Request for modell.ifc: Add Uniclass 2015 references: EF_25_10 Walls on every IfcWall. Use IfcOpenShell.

First a look at what the model holds.

```python
import ifcopenshell

model = ifcopenshell.open("modell.ifc")
print(model.schema)
print("classifications:", [c.Name for c in model.by_type("IfcClassification")])
for ifc_class in ("IfcDoor", "IfcRoof", "IfcStair", "IfcWall", "IfcWindow"):
    print(ifc_class, len(model.by_type(ifc_class)))
```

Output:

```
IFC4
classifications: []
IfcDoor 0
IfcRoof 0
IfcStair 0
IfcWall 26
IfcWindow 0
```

```python
import ifcopenshell
import ifcopenshell.api.classification

model = ifcopenshell.open("modell.ifc")

system = ifcopenshell.api.classification.add_classification(model, classification="Uniclass 2015")

codes = {
    "IfcWall": ("EF_25_10", "Walls"),
}
for ifc_class, (code, name) in codes.items():
    products = model.by_type(ifc_class)
    ifcopenshell.api.classification.add_reference(
        model, products=products, classification=system, identification=code, name=name
    )
    print(code, len(products))

model.write("modell_v2.ifc")
```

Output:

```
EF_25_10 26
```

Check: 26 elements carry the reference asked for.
